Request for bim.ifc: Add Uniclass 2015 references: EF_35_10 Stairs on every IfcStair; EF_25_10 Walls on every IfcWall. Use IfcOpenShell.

First a look at what the model holds.

```python
import ifcopenshell

model = ifcopenshell.open("bim.ifc")
print(model.schema)
print("classifications:", [c.Name for c in model.by_type("IfcClassification")])
for ifc_class in ("IfcDoor", "IfcRoof", "IfcStair", "IfcWall", "IfcWindow"):
    print(ifc_class, len(model.by_type(ifc_class)))
```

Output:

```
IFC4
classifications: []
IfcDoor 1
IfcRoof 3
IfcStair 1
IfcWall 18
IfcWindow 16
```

```python
import ifcopenshell
import ifcopenshell.api.classification

model = ifcopenshell.open("bim.ifc")

system = ifcopenshell.api.classification.add_classification(model, classification="Uniclass 2015")

codes = {
    "IfcStair": ("EF_35_10", "Stairs"),
    "IfcWall": ("EF_25_10", "Walls"),
}
for ifc_class, (code, name) in codes.items():
    products = model.by_type(ifc_class)
    ifcopenshell.api.classification.add_reference(
        model, products=products, classification=system, identification=code, name=name
    )
    print(code, len(products))

model.write("bim_edited.ifc")
```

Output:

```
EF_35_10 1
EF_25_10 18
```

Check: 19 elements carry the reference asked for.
